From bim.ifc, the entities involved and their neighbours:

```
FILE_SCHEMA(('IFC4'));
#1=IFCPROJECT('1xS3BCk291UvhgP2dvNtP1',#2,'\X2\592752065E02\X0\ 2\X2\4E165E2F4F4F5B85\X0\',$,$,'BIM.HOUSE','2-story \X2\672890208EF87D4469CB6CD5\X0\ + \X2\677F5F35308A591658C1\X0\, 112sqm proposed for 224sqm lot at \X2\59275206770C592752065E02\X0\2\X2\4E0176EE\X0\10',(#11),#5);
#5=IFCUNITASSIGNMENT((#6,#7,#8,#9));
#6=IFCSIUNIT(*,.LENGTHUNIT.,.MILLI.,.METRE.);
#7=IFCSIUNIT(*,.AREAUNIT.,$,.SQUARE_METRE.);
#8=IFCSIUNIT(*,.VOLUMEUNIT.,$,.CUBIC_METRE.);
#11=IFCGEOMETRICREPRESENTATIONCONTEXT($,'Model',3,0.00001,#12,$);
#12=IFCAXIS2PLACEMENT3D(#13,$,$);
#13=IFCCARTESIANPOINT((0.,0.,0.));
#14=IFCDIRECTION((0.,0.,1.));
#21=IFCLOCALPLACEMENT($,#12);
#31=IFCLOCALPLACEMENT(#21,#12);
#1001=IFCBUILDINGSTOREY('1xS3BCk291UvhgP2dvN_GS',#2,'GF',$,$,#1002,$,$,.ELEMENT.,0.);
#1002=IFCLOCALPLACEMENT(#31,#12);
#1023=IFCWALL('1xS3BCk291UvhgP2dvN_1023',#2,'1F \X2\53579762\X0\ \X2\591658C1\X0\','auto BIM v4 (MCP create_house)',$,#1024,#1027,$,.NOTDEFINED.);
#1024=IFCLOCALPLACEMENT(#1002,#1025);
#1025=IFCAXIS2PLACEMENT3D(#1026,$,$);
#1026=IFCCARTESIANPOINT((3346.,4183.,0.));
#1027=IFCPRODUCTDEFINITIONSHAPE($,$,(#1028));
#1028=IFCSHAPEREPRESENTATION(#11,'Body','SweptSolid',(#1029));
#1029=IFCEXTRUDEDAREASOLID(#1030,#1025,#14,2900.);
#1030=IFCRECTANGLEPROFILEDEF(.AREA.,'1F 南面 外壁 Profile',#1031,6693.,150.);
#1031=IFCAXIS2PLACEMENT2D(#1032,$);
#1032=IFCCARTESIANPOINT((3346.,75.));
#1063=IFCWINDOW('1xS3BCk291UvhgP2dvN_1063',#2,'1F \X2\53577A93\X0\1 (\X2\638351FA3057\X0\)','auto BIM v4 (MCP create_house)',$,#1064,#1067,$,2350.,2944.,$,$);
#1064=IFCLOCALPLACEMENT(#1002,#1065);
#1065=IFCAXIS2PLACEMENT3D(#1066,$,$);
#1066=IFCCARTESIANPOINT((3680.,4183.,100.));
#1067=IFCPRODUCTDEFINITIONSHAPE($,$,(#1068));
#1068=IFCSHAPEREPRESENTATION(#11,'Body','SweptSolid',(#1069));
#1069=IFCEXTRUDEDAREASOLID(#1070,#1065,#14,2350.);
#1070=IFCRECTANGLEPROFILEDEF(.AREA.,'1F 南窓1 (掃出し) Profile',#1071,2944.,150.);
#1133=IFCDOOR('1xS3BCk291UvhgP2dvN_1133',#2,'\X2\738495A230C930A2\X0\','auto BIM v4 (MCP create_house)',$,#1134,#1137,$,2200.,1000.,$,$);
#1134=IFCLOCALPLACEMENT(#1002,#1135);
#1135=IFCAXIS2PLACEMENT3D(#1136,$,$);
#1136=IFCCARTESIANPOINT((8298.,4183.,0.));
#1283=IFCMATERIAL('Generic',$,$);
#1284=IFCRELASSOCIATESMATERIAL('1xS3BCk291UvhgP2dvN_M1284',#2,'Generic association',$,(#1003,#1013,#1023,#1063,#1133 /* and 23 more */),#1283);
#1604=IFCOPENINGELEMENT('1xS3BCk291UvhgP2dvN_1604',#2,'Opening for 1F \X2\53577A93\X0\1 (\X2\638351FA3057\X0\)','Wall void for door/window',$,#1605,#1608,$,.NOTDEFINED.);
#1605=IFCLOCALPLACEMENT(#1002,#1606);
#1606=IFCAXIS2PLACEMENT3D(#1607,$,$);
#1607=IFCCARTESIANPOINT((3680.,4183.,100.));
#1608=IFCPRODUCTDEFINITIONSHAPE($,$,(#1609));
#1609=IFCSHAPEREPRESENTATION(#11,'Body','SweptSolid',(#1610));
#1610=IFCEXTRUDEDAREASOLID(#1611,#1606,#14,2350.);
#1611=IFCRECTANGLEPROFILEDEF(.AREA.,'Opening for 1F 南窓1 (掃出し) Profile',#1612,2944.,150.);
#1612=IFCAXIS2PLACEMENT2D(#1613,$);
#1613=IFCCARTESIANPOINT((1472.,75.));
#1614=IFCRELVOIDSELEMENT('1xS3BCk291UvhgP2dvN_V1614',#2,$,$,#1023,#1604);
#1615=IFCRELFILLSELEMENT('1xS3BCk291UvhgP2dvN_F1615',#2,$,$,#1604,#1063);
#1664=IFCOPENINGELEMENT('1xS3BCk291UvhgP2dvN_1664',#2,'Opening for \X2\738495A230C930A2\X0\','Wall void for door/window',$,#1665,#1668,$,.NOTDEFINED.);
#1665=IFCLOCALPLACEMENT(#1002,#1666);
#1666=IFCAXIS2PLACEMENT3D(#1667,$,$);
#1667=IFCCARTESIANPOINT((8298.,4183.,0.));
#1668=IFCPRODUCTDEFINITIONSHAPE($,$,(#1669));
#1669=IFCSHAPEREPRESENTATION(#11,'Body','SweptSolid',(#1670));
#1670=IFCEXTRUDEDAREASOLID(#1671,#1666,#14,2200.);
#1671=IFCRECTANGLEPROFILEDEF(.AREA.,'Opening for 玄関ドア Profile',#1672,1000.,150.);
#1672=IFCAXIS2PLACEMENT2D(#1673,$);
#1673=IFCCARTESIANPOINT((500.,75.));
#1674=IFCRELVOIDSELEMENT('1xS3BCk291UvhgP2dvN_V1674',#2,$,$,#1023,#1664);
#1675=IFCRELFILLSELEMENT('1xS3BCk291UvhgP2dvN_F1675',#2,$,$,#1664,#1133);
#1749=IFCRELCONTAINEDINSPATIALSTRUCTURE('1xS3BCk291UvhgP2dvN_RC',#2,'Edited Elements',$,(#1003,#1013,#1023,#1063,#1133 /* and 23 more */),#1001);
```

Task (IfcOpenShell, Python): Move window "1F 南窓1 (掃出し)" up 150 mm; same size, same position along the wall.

```python
import numpy as np
import ifcopenshell
import ifcopenshell.api.geometry
import ifcopenshell.util.placement
import ifcopenshell.util.unit

model = ifcopenshell.open("bim.ifc")
unit_scale = ifcopenshell.util.unit.calculate_unit_scale(model)

window = model.by_guid("1xS3BCk291UvhgP2dvN_1063")
opening = window.FillsVoids[0].RelatingOpeningElement
dz = 150.0

shift = np.array([0.0, 0.0, dz])
# The window is not placed relative to its opening, so move both.
for product in (opening, window):
    matrix = ifcopenshell.util.placement.get_local_placement(product.ObjectPlacement)
    matrix[:3, 3] += shift
    ifcopenshell.api.geometry.edit_object_placement(model, product=product, matrix=matrix, is_si=False)

print(f"moved by {dz * unit_scale:+.3f} m")

model.write("bim_edited.ifc")
```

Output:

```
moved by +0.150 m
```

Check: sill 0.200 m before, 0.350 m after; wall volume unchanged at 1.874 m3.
